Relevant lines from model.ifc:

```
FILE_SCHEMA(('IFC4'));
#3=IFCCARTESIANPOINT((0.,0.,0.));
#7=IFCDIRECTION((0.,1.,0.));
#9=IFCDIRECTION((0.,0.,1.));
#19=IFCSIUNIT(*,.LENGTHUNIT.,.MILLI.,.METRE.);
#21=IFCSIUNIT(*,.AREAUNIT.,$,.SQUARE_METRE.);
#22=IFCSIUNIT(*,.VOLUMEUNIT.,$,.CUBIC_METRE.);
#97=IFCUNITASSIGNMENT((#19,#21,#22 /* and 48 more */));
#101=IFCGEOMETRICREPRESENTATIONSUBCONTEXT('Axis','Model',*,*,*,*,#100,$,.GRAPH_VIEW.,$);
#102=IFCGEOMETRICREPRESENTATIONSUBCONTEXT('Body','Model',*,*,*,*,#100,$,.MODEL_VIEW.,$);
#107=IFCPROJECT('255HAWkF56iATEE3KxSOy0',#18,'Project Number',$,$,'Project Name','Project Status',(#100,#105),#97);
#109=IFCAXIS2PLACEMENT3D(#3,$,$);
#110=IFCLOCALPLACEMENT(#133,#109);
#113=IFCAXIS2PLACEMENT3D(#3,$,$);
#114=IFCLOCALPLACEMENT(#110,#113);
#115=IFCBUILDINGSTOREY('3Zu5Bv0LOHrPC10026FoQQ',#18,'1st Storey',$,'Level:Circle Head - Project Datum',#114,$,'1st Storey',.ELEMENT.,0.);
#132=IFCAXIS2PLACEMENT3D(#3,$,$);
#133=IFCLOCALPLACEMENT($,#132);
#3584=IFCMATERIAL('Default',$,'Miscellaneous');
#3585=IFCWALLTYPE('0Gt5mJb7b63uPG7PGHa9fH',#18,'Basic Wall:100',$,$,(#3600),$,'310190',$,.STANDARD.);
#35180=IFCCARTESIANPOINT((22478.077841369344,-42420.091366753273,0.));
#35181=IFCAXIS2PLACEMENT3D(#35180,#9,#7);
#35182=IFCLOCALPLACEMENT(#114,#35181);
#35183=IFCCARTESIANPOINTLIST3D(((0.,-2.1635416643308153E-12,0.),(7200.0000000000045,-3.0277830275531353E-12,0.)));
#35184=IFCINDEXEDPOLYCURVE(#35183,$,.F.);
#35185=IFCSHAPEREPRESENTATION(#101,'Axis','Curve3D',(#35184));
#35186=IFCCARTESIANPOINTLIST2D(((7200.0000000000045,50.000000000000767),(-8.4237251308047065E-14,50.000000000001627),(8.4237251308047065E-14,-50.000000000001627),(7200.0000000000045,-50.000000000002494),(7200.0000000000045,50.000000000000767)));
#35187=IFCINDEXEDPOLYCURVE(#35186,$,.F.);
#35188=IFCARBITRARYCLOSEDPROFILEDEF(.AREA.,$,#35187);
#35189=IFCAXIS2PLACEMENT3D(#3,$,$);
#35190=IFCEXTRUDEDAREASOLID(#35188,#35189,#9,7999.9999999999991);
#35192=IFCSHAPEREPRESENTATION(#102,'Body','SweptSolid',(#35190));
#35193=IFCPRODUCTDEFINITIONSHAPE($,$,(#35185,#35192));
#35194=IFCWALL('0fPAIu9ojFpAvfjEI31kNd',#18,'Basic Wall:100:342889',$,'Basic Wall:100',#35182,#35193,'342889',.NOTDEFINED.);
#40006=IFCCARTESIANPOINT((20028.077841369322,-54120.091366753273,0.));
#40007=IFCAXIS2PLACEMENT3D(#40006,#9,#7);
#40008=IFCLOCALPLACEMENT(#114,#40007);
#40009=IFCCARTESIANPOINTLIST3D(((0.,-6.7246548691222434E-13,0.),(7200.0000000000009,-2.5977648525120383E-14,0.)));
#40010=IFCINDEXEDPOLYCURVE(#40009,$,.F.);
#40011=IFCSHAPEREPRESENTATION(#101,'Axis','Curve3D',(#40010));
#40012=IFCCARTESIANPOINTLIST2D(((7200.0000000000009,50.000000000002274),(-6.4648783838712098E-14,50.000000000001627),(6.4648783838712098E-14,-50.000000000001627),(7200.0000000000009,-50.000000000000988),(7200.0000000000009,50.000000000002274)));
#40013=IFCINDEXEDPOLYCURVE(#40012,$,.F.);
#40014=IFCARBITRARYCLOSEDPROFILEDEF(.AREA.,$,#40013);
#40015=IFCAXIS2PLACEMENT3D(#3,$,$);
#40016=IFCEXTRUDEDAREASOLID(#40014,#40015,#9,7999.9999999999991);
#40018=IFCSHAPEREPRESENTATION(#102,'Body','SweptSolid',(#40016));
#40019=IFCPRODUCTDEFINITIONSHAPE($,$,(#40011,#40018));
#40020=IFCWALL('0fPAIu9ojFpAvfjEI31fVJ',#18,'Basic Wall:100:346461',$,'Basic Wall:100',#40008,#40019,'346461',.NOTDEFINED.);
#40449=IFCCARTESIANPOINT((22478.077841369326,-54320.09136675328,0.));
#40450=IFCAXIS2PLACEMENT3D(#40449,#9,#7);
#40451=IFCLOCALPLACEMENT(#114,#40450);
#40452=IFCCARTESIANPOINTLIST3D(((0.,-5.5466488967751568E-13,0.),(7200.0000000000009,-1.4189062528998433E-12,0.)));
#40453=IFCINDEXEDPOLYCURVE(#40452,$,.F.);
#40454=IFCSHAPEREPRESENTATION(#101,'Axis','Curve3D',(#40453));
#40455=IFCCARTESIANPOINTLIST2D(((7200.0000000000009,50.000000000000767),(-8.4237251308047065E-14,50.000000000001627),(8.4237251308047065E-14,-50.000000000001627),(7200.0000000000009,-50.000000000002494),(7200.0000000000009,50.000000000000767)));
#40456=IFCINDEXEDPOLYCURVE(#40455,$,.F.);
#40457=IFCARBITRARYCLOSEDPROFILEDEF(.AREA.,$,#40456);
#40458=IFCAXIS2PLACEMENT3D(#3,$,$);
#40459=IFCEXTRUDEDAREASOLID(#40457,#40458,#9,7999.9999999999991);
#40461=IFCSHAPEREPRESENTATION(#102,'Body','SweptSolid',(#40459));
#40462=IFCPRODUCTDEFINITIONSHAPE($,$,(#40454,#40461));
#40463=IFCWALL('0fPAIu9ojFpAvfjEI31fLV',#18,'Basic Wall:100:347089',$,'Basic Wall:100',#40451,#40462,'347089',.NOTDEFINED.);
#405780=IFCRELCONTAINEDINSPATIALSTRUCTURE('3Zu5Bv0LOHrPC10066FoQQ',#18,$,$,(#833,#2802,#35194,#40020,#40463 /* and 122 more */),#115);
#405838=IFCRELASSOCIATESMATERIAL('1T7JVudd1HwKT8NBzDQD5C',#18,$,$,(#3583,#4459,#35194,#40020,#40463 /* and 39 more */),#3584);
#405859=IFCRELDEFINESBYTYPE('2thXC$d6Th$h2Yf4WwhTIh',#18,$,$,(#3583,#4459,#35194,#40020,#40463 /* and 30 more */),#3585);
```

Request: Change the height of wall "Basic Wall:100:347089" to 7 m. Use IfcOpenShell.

```python
import ifcopenshell
import ifcopenshell.geom
import ifcopenshell.util.representation
import ifcopenshell.util.shape
import ifcopenshell.util.unit

model = ifcopenshell.open("model.ifc")
unit_scale = ifcopenshell.util.unit.calculate_unit_scale(model)
settings = ifcopenshell.geom.settings()


def volume(element):
    """Net volume in cubic metres, openings subtracted."""
    shape = ifcopenshell.geom.create_shape(settings, element)
    return ifcopenshell.util.shape.get_volume(shape.geometry)


wall = model.by_guid("0fPAIu9ojFpAvfjEI31fLV")
before = volume(wall)

body = ifcopenshell.util.representation.get_representation(wall, "Model", "Body")
solid = body.Items[0]
old_height = solid.Depth
solid.Depth = 7 / unit_scale
after = volume(wall)

print(f"height {old_height:g} -> {solid.Depth:g}, volume {before:.3f} -> {after:.3f} m3")

model.write("model_updated.ifc")
```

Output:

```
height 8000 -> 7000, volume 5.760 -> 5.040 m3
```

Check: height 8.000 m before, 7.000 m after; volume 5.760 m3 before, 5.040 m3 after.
